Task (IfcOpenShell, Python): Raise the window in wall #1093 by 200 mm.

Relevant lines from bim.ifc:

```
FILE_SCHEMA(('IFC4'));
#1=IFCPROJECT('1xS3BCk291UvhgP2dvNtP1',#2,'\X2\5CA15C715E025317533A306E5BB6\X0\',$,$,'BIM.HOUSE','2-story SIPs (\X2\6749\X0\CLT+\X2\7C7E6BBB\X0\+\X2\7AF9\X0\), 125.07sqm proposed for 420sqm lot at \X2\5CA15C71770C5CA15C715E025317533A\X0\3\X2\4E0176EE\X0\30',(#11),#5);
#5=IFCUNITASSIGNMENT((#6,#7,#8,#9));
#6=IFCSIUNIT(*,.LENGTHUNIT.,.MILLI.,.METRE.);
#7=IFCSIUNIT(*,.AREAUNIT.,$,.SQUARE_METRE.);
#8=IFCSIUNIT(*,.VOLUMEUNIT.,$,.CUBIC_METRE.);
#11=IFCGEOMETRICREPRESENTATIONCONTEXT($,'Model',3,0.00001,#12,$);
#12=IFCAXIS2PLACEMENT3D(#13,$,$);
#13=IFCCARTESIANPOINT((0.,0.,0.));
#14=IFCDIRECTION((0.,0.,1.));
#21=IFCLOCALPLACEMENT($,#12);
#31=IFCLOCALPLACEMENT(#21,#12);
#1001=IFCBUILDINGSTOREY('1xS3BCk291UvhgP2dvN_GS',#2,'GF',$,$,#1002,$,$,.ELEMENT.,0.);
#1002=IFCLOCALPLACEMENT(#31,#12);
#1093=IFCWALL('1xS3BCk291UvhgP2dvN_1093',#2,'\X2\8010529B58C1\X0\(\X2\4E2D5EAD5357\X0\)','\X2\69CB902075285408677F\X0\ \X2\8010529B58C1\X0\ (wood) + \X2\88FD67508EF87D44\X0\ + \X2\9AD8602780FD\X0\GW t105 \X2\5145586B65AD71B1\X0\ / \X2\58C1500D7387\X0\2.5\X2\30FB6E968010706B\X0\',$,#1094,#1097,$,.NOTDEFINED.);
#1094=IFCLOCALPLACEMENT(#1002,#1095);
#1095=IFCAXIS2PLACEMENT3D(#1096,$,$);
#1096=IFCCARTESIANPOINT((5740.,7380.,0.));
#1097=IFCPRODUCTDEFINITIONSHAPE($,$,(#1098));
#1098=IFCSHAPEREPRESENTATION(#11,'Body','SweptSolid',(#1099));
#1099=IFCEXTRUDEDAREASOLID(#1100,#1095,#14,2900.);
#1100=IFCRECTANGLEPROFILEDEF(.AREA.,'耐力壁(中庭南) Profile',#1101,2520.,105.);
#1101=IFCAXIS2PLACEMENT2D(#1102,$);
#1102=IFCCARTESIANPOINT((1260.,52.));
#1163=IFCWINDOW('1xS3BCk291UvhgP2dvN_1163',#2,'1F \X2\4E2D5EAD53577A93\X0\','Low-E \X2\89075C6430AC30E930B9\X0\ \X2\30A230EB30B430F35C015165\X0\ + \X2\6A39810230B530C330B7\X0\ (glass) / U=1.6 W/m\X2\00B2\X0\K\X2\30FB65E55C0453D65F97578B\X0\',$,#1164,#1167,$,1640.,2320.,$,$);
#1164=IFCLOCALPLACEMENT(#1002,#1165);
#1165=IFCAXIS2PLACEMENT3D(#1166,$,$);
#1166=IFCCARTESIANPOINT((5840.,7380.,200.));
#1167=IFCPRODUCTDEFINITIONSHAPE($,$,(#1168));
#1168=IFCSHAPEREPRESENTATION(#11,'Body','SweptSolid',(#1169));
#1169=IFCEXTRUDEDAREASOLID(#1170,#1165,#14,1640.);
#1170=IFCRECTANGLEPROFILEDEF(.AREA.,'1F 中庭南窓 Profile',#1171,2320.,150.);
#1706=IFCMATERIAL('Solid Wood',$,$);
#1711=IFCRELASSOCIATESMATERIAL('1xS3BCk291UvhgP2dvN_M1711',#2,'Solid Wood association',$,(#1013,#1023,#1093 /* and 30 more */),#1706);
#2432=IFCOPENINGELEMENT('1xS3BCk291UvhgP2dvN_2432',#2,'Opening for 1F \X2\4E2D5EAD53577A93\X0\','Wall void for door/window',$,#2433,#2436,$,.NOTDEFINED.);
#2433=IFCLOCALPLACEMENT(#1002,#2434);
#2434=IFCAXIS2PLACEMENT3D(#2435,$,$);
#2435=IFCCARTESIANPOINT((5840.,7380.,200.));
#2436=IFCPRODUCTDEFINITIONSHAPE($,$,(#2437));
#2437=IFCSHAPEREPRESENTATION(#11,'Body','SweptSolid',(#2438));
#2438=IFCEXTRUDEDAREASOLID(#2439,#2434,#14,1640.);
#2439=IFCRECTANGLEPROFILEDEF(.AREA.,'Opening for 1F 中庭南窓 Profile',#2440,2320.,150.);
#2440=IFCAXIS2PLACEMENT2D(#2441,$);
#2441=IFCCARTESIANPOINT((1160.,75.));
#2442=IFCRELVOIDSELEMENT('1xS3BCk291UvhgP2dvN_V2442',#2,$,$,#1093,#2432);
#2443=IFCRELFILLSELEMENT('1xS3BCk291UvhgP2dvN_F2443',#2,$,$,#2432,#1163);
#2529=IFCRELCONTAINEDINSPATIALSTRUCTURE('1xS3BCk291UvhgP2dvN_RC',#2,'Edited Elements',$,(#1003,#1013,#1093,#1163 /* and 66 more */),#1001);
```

```python
import numpy as np
import ifcopenshell
import ifcopenshell.api.geometry
import ifcopenshell.util.placement
import ifcopenshell.util.unit

model = ifcopenshell.open("bim.ifc")
unit_scale = ifcopenshell.util.unit.calculate_unit_scale(model)

window = model.by_guid("1xS3BCk291UvhgP2dvN_1163")
opening = window.FillsVoids[0].RelatingOpeningElement
dz = 0.2 / unit_scale

shift = np.array([0.0, 0.0, dz])
# The window is not placed relative to its opening, so move both.
for product in (opening, window):
    matrix = ifcopenshell.util.placement.get_local_placement(product.ObjectPlacement)
    matrix[:3, 3] += shift
    ifcopenshell.api.geometry.edit_object_placement(model, product=product, matrix=matrix, is_si=False)

print(f"moved by {dz * unit_scale:+.3f} m")

model.write("bim_rev.ifc")
```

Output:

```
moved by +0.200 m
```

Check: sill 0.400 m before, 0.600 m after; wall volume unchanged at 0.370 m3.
